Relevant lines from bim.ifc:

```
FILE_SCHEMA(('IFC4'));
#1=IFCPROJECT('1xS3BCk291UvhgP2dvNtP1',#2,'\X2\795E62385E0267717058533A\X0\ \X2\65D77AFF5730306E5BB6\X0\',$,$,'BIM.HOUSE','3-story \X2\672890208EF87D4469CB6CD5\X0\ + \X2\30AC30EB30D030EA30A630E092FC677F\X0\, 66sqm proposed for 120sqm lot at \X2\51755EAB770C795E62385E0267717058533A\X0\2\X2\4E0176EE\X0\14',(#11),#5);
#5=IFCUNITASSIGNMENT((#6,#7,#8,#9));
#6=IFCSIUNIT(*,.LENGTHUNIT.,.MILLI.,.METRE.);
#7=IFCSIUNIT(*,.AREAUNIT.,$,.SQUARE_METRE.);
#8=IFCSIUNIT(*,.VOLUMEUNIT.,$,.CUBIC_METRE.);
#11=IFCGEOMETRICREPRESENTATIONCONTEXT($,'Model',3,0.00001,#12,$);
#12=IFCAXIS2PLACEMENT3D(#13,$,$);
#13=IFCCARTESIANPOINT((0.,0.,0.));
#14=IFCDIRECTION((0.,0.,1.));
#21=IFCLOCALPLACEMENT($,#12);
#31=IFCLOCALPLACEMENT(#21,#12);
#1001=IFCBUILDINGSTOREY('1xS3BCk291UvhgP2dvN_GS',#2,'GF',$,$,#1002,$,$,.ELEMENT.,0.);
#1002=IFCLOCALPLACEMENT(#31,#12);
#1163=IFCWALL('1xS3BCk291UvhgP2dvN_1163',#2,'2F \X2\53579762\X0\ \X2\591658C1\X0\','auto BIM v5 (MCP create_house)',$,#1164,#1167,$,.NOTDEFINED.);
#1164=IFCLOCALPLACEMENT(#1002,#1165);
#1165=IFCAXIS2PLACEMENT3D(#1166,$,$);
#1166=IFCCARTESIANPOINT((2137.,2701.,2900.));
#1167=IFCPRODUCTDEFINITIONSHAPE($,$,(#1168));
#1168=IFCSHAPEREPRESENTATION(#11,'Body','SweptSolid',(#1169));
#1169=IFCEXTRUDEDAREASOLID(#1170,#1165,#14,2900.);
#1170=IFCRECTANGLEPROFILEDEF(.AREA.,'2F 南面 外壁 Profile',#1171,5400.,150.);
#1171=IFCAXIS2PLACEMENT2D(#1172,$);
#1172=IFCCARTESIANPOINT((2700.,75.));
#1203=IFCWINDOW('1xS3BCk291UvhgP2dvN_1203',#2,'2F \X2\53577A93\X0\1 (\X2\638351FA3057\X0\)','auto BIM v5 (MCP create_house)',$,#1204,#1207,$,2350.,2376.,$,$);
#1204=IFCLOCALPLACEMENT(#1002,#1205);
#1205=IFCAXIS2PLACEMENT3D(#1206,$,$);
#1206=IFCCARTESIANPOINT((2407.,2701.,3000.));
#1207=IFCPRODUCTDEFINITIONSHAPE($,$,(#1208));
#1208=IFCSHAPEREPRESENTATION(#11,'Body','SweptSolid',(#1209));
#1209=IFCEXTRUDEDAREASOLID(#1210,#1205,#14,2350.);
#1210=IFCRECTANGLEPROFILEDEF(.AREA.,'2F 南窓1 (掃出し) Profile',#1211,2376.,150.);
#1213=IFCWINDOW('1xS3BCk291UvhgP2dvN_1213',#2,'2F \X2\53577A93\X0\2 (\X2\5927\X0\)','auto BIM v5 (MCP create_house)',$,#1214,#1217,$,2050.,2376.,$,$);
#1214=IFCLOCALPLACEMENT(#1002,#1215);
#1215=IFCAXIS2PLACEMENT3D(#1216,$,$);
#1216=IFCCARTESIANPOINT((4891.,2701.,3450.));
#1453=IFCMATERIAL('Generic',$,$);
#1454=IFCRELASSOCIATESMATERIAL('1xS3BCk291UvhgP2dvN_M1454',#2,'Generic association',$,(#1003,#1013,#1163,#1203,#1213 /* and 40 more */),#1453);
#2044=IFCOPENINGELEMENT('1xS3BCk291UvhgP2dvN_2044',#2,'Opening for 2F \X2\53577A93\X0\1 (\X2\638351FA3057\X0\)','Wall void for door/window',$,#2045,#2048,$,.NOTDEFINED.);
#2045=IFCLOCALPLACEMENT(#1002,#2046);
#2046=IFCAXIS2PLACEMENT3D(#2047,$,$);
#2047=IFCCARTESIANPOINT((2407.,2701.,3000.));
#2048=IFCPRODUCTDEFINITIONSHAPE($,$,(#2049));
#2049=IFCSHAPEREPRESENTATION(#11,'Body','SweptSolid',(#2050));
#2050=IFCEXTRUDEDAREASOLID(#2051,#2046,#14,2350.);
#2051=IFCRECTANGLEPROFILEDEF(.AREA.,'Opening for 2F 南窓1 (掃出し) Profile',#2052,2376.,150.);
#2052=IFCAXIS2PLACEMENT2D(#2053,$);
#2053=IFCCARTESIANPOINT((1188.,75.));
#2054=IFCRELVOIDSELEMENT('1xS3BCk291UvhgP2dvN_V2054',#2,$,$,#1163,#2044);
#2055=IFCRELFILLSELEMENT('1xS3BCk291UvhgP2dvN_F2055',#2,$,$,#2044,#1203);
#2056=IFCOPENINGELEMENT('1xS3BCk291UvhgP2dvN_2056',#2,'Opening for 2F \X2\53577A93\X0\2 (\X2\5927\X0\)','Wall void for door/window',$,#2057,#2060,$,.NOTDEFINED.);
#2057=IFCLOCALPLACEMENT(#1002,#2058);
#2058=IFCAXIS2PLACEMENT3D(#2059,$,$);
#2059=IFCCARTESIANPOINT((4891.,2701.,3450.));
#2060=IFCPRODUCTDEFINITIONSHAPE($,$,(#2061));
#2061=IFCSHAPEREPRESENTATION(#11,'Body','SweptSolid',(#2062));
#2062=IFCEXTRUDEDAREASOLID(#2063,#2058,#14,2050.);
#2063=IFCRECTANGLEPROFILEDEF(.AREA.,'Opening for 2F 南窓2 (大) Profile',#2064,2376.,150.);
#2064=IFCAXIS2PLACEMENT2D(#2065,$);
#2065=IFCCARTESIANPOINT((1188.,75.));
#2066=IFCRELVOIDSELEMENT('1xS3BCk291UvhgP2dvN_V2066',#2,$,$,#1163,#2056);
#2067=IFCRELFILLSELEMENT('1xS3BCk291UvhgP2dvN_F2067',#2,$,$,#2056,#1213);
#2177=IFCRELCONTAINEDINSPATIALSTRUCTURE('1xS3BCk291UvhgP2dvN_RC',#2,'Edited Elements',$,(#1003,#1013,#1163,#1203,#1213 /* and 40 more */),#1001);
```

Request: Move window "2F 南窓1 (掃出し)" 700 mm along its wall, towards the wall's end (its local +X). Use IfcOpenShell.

```python
import ifcopenshell
import ifcopenshell.api.geometry
import ifcopenshell.util.placement
import ifcopenshell.util.unit

model = ifcopenshell.open("bim.ifc")
unit_scale = ifcopenshell.util.unit.calculate_unit_scale(model)

window = model.by_guid("1xS3BCk291UvhgP2dvN_1203")
opening = window.FillsVoids[0].RelatingOpeningElement
wall = opening.VoidsElements[0].RelatingBuildingElement

wall_matrix = ifcopenshell.util.placement.get_local_placement(wall.ObjectPlacement)
shift = wall_matrix[:3, 0] * 0.7 / unit_scale
before = ifcopenshell.util.placement.get_local_placement(window.ObjectPlacement)[:3, 3].copy()

# The window is not placed relative to its opening, so move both.
for product in (opening, window):
    matrix = ifcopenshell.util.placement.get_local_placement(product.ObjectPlacement)
    matrix[:3, 3] += shift
    ifcopenshell.api.geometry.edit_object_placement(model, product=product, matrix=matrix, is_si=False)

after = ifcopenshell.util.placement.get_local_placement(window.ObjectPlacement)[:3, 3]
print("window moved by", (after - before).round(3) + 0.0)

model.write("bim_updated.ifc")
```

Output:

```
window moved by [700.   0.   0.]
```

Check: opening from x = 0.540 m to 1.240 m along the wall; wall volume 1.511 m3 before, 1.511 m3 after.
